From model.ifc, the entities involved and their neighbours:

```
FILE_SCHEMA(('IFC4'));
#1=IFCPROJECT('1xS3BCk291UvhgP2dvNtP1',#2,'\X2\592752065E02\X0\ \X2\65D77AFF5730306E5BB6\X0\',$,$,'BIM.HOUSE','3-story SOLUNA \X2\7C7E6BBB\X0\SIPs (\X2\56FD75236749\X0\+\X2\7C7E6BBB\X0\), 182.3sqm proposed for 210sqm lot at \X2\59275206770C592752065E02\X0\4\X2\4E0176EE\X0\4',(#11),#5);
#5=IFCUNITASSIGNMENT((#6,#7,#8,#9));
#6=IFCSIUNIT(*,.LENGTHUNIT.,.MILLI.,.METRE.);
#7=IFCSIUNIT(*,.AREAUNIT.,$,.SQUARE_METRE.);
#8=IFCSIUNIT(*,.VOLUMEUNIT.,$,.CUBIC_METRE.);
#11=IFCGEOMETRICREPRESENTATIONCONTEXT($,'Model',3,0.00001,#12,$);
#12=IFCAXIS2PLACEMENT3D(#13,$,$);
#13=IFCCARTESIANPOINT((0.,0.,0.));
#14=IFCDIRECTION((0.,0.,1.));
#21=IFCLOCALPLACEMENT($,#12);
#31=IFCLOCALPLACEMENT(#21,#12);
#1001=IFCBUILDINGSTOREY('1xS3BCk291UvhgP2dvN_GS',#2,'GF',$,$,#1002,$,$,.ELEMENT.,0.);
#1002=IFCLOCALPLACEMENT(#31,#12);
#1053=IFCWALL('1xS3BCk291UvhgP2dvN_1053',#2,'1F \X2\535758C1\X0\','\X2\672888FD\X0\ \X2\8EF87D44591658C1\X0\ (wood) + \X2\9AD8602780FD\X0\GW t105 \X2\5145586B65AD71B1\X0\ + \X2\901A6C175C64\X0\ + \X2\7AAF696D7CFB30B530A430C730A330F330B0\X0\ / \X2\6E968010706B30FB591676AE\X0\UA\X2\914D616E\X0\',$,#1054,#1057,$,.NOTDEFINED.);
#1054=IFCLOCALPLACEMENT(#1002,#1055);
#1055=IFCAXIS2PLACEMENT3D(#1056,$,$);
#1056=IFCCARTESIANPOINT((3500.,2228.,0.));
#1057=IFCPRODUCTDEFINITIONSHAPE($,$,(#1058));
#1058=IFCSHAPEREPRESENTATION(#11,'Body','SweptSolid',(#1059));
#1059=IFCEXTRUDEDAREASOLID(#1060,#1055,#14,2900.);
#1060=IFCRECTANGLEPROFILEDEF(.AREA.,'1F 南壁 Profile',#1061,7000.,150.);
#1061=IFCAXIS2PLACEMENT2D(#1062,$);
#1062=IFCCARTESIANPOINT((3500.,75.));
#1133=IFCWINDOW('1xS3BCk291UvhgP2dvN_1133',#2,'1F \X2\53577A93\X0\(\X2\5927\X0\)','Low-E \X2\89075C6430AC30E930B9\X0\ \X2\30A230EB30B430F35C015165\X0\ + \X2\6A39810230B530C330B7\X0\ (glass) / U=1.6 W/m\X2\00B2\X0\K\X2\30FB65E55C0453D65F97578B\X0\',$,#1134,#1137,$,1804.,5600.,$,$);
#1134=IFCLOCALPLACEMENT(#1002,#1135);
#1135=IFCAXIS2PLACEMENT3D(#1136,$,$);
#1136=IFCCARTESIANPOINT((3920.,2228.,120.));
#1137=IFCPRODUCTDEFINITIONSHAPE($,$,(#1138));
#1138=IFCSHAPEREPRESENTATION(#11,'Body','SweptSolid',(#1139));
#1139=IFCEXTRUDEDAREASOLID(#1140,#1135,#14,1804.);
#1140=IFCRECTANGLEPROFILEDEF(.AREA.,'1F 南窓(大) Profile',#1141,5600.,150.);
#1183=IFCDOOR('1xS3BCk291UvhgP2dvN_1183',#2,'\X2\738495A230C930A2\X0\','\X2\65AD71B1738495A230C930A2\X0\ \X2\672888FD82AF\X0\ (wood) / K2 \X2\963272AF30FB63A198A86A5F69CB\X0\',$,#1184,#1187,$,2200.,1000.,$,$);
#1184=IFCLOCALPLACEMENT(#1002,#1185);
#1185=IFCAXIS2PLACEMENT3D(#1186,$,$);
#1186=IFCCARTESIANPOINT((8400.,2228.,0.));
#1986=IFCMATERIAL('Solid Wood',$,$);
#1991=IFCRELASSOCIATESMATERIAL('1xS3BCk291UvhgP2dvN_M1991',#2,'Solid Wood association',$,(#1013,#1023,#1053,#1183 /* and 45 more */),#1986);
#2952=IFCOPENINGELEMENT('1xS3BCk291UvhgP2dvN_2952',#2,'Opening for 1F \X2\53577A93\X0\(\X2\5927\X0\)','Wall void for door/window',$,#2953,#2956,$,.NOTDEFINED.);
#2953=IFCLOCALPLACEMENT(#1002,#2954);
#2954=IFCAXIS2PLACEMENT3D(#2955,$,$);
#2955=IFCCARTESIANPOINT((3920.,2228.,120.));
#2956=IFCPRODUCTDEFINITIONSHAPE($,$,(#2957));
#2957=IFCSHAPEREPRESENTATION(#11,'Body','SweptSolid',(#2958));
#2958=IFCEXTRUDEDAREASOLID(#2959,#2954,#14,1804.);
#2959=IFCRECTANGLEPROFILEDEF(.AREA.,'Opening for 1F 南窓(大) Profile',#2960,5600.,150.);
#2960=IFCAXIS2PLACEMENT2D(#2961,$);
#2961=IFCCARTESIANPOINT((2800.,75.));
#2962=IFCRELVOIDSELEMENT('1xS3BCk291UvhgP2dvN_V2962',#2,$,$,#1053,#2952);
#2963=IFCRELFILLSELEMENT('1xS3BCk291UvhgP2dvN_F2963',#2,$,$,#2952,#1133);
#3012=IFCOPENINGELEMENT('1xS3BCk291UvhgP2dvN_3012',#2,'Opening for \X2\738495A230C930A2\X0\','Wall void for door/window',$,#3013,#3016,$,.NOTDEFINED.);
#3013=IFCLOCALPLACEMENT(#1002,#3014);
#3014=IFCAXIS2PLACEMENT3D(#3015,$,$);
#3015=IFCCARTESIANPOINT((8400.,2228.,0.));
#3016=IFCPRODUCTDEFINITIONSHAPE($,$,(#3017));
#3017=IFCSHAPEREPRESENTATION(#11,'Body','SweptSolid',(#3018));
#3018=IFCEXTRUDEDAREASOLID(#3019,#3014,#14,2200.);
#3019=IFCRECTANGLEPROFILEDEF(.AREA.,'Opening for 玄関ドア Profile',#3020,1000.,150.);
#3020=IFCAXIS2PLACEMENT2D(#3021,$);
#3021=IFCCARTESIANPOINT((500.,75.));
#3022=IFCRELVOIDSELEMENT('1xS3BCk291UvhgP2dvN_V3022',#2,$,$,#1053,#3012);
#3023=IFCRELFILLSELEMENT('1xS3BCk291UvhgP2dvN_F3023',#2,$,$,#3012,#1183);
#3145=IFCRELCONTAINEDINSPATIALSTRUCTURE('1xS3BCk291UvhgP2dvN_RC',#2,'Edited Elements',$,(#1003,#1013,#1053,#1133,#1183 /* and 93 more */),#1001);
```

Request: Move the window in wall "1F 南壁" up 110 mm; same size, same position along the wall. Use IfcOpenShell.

```python
import numpy as np
import ifcopenshell
import ifcopenshell.api.geometry
import ifcopenshell.util.placement
import ifcopenshell.util.unit

model = ifcopenshell.open("model.ifc")
unit_scale = ifcopenshell.util.unit.calculate_unit_scale(model)

window = model.by_guid("1xS3BCk291UvhgP2dvN_1133")
opening = window.FillsVoids[0].RelatingOpeningElement
dz = 110.0

shift = np.array([0.0, 0.0, dz])
# The window is not placed relative to its opening, so move both.
for product in (opening, window):
    matrix = ifcopenshell.util.placement.get_local_placement(product.ObjectPlacement)
    matrix[:3, 3] += shift
    ifcopenshell.api.geometry.edit_object_placement(model, product=product, matrix=matrix, is_si=False)

print(f"moved by {dz * unit_scale:+.3f} m")

model.write("model_updated.ifc")
```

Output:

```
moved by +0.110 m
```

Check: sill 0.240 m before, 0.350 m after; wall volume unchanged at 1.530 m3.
